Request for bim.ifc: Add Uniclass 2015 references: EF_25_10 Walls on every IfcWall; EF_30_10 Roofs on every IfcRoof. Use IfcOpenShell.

First a look at what the model holds.

```python
import ifcopenshell

model = ifcopenshell.open("bim.ifc")
print(model.schema)
print("classifications:", [c.Name for c in model.by_type("IfcClassification")])
for ifc_class in ("IfcDoor", "IfcRoof", "IfcStair", "IfcWall", "IfcWindow"):
    print(ifc_class, len(model.by_type(ifc_class)))
```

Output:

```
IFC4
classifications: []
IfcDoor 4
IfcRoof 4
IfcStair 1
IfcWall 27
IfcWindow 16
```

```python
import ifcopenshell
import ifcopenshell.api.classification

model = ifcopenshell.open("bim.ifc")

system = ifcopenshell.api.classification.add_classification(model, classification="Uniclass 2015")

codes = {
    "IfcWall": ("EF_25_10", "Walls"),
    "IfcRoof": ("EF_30_10", "Roofs"),
}
for ifc_class, (code, name) in codes.items():
    products = model.by_type(ifc_class)
    ifcopenshell.api.classification.add_reference(
        model, products=products, classification=system, identification=code, name=name
    )
    print(code, len(products))

model.write("bim_rev.ifc")
```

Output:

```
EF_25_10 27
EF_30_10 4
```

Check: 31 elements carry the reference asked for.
